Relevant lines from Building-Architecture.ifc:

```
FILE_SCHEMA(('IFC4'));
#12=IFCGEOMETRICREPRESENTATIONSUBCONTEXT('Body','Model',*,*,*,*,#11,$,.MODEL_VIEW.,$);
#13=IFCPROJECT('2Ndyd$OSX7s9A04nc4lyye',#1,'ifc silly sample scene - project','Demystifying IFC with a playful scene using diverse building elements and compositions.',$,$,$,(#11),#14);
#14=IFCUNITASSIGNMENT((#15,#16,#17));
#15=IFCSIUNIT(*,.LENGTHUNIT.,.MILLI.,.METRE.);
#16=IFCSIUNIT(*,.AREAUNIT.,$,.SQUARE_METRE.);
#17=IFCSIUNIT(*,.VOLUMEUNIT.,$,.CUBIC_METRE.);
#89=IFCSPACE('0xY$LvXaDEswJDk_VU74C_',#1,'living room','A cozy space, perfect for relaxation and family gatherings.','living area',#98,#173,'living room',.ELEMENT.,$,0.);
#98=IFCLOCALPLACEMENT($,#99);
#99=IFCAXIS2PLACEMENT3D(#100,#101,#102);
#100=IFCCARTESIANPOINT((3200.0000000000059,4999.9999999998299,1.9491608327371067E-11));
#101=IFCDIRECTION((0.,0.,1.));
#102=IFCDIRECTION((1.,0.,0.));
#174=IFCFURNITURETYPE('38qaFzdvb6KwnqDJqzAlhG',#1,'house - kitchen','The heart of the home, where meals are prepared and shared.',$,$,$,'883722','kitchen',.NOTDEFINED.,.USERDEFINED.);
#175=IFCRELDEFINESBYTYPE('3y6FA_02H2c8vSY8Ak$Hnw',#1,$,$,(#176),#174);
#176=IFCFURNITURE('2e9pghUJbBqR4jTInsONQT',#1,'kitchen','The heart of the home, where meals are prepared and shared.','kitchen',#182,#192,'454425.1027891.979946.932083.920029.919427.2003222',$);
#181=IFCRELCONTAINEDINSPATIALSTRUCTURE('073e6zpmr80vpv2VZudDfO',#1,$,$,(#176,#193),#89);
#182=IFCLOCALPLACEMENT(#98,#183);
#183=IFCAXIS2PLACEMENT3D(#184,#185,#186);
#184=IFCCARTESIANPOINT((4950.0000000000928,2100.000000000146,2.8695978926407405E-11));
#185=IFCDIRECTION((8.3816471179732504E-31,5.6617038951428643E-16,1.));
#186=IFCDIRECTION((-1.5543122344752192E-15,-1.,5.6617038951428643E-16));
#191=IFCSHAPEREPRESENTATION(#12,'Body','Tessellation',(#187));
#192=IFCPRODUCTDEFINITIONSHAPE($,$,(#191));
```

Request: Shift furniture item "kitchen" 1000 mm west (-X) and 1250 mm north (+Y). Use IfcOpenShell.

```python
import ifcopenshell
import ifcopenshell.api.geometry
import ifcopenshell.util.placement
import ifcopenshell.util.unit

model = ifcopenshell.open("Building-Architecture.ifc")
unit_scale = ifcopenshell.util.unit.calculate_unit_scale(model)

item = model.by_guid("2e9pghUJbBqR4jTInsONQT")
matrix = ifcopenshell.util.placement.get_local_placement(item.ObjectPlacement)
matrix[0, 3] -= 1 / unit_scale
matrix[1, 3] += 1.25 / unit_scale
ifcopenshell.api.geometry.edit_object_placement(model, product=item, matrix=matrix, is_si=False)

print(ifcopenshell.util.placement.get_local_placement(item.ObjectPlacement).round(3) + 0.0)

model.write("Building-Architecture-out.ifc")
```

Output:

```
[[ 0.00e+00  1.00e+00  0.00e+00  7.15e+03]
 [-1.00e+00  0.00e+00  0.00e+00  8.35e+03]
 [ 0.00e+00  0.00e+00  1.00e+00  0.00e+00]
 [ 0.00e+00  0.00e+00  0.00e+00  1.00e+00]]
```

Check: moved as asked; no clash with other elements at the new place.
